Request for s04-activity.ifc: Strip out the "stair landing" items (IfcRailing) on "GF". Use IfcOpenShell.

First a look at what the model holds.

```python
import ifcopenshell
import ifcopenshell.util.element

model = ifcopenshell.open("s04-activity.ifc")
print(model.schema)
storey = next(s for s in model.by_type("IfcBuildingStorey") if s.Name == "GF")
railings = [e for e in ifcopenshell.util.element.get_decomposition(storey) if e.is_a("IfcRailing")]
seen = {}
for e in railings:
    element_type = ifcopenshell.util.element.get_type(e)
    name = element_type.Name if element_type not in (None, e) else None
    seen[name] = seen.get(name, 0) + 1
for name, count in sorted(seen.items(), key=str):
    print(count, "x", name)
```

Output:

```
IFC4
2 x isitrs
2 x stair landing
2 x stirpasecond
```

```python
import ifcopenshell
import ifcopenshell.api.root
import ifcopenshell.util.element

model = ifcopenshell.open("s04-activity.ifc")

storey = next(s for s in model.by_type("IfcBuildingStorey") if s.Name == "GF")
railings = [e for e in ifcopenshell.util.element.get_decomposition(storey) if e.is_a("IfcRailing")]
targets = [e for e in railings if (t := ifcopenshell.util.element.get_type(e)) not in (None, e) and t.Name == "stair landing"]

for e in targets:
    ifcopenshell.api.root.remove_product(model, product=e)
print(len(targets), "removed")

model.write("s04-activity-out.ifc")
```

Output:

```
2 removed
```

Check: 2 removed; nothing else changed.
